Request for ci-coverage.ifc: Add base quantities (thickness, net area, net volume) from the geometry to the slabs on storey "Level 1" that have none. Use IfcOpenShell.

First a look at what the model holds.

```python
import ifcopenshell
import ifcopenshell.util.element
import ifcopenshell.util.unit

model = ifcopenshell.open("ci-coverage.ifc")
print(model.schema)
for unit_type in ("LENGTHUNIT", "AREAUNIT", "VOLUMEUNIT"):
    print(unit_type, ifcopenshell.util.unit.calculate_unit_scale(model, unit_type))
storey = next(s for s in model.by_type("IfcBuildingStorey") if s.Name == "Level 1")
slabs = [e for e in ifcopenshell.util.element.get_decomposition(storey) if e.is_a("IfcSlab")]
for e in sorted(slabs, key=lambda e: e.id()):
    print(e.id(), e.is_a(), e.Name, list(ifcopenshell.util.element.get_psets(e, qtos_only=True)), sep=" | ")
```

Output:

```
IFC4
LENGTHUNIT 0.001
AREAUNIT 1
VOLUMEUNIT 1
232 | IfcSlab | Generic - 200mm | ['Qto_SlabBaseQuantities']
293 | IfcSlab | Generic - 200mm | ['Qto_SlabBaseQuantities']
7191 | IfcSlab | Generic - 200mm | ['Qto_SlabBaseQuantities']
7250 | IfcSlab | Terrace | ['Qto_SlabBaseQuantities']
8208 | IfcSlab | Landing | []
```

```python
import ifcopenshell
import ifcopenshell.api.pset
import ifcopenshell.geom
import ifcopenshell.util.element
import ifcopenshell.util.shape
import ifcopenshell.util.unit

model = ifcopenshell.open("ci-coverage.ifc")
unit_scale = ifcopenshell.util.unit.calculate_unit_scale(model)
area_scale = ifcopenshell.util.unit.calculate_unit_scale(model, "AREAUNIT")
volume_scale = ifcopenshell.util.unit.calculate_unit_scale(model, "VOLUMEUNIT")
settings = ifcopenshell.geom.settings()

storey = next(s for s in model.by_type("IfcBuildingStorey") if s.Name == "Level 1")
slabs = [e for e in ifcopenshell.util.element.get_decomposition(storey) if e.is_a("IfcSlab")]

for e in sorted(slabs, key=lambda e: e.id()):
    if ifcopenshell.util.element.get_psets(e, qtos_only=True, should_inherit=False):
        continue
    # Geometry comes back in metres, in the element's own axes.
    shape = ifcopenshell.geom.create_shape(settings, e)
    values = {
        "Width": ifcopenshell.util.shape.get_z(shape.geometry) / unit_scale,
        "NetArea": ifcopenshell.util.shape.get_footprint_area(shape.geometry) / area_scale,
        "NetVolume": ifcopenshell.util.shape.get_volume(shape.geometry) / volume_scale,
    }
    qto = ifcopenshell.api.pset.add_qto(model, product=e, name="Qto_SlabBaseQuantities")
    ifcopenshell.api.pset.edit_qto(model, qto=qto, properties=values)
    print(e.id(), {k: round(v, 3) for k, v in values.items()})

model.write("ci-coverage_rev.ifc")
```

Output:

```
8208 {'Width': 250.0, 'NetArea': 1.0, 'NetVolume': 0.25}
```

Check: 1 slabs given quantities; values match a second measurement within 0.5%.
